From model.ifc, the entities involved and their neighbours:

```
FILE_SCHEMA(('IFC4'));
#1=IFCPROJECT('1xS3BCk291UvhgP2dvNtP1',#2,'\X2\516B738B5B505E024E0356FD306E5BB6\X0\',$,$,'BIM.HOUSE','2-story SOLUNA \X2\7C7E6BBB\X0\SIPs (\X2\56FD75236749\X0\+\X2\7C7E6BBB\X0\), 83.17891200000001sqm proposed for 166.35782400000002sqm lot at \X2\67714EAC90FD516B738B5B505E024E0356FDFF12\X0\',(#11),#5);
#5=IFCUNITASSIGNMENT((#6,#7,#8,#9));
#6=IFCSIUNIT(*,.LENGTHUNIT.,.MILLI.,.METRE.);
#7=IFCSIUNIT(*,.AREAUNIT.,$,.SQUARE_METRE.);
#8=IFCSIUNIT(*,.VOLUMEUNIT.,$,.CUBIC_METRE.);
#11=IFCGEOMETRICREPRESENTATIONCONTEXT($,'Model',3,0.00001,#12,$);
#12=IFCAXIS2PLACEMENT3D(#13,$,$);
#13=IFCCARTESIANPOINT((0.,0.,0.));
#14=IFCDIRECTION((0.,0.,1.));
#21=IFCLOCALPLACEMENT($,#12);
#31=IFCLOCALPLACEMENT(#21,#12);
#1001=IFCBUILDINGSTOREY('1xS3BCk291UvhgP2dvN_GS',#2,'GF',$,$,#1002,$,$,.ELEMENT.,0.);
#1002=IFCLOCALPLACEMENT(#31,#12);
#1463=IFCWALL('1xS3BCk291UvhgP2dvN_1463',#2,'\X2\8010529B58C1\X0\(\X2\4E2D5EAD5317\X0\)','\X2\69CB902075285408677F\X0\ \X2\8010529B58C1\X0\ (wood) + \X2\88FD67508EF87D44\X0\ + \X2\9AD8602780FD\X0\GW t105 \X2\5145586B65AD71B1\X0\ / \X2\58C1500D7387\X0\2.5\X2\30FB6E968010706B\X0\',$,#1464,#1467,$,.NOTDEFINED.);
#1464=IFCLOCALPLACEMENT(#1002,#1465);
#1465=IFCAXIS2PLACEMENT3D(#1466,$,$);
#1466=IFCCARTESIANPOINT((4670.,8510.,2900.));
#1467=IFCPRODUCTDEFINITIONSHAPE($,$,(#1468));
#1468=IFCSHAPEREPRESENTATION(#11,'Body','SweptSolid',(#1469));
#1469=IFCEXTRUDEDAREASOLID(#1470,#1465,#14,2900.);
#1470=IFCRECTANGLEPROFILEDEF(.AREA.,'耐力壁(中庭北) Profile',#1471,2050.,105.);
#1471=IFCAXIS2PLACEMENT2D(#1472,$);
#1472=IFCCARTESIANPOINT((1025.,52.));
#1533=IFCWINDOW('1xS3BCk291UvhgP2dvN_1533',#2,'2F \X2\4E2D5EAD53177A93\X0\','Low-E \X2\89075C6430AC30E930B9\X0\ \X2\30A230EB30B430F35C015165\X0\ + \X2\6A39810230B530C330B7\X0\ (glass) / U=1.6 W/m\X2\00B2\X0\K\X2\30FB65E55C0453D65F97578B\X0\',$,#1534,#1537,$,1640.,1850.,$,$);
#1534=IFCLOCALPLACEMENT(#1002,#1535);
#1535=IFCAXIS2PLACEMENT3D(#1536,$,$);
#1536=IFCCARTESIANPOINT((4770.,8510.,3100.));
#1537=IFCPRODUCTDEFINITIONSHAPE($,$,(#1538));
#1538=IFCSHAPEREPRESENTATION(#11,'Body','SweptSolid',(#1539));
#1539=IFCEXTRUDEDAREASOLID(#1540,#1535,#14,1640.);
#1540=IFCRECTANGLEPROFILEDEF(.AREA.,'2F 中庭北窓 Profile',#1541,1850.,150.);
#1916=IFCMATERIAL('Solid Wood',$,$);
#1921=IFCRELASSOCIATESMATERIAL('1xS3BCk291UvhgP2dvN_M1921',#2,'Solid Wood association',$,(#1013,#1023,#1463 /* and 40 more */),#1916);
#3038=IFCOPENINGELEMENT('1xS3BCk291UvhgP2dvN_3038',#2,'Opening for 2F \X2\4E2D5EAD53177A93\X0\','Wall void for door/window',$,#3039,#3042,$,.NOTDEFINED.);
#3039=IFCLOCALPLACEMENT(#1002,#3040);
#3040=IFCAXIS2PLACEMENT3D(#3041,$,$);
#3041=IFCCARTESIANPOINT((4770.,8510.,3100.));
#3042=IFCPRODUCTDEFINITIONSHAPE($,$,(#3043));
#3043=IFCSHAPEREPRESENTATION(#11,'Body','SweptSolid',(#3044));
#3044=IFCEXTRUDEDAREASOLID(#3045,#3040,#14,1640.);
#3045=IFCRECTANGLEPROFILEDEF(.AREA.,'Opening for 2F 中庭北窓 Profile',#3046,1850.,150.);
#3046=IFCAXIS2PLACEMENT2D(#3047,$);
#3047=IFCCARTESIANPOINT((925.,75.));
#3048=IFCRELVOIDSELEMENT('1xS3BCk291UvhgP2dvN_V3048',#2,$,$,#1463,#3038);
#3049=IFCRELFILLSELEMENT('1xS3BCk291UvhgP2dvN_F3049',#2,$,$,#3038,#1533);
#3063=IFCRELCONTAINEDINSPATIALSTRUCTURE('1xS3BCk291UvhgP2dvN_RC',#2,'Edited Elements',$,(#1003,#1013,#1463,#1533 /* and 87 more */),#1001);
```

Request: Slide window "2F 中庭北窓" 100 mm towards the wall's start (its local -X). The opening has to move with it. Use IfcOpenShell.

```python
import ifcopenshell
import ifcopenshell.api.geometry
import ifcopenshell.util.placement
import ifcopenshell.util.unit

model = ifcopenshell.open("model.ifc")
unit_scale = ifcopenshell.util.unit.calculate_unit_scale(model)

window = model.by_guid("1xS3BCk291UvhgP2dvN_1533")
opening = window.FillsVoids[0].RelatingOpeningElement
wall = opening.VoidsElements[0].RelatingBuildingElement

wall_matrix = ifcopenshell.util.placement.get_local_placement(wall.ObjectPlacement)
shift = wall_matrix[:3, 0] * -0.1 / unit_scale
before = ifcopenshell.util.placement.get_local_placement(window.ObjectPlacement)[:3, 3].copy()

# The window is not placed relative to its opening, so move both.
for product in (opening, window):
    matrix = ifcopenshell.util.placement.get_local_placement(product.ObjectPlacement)
    matrix[:3, 3] += shift
    ifcopenshell.api.geometry.edit_object_placement(model, product=product, matrix=matrix, is_si=False)

after = ifcopenshell.util.placement.get_local_placement(window.ObjectPlacement)[:3, 3]
print("window moved by", (after - before).round(3) + 0.0)

model.write("model_rev.ifc")
```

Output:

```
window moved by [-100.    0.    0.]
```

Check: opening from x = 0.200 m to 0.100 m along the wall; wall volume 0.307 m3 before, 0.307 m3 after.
